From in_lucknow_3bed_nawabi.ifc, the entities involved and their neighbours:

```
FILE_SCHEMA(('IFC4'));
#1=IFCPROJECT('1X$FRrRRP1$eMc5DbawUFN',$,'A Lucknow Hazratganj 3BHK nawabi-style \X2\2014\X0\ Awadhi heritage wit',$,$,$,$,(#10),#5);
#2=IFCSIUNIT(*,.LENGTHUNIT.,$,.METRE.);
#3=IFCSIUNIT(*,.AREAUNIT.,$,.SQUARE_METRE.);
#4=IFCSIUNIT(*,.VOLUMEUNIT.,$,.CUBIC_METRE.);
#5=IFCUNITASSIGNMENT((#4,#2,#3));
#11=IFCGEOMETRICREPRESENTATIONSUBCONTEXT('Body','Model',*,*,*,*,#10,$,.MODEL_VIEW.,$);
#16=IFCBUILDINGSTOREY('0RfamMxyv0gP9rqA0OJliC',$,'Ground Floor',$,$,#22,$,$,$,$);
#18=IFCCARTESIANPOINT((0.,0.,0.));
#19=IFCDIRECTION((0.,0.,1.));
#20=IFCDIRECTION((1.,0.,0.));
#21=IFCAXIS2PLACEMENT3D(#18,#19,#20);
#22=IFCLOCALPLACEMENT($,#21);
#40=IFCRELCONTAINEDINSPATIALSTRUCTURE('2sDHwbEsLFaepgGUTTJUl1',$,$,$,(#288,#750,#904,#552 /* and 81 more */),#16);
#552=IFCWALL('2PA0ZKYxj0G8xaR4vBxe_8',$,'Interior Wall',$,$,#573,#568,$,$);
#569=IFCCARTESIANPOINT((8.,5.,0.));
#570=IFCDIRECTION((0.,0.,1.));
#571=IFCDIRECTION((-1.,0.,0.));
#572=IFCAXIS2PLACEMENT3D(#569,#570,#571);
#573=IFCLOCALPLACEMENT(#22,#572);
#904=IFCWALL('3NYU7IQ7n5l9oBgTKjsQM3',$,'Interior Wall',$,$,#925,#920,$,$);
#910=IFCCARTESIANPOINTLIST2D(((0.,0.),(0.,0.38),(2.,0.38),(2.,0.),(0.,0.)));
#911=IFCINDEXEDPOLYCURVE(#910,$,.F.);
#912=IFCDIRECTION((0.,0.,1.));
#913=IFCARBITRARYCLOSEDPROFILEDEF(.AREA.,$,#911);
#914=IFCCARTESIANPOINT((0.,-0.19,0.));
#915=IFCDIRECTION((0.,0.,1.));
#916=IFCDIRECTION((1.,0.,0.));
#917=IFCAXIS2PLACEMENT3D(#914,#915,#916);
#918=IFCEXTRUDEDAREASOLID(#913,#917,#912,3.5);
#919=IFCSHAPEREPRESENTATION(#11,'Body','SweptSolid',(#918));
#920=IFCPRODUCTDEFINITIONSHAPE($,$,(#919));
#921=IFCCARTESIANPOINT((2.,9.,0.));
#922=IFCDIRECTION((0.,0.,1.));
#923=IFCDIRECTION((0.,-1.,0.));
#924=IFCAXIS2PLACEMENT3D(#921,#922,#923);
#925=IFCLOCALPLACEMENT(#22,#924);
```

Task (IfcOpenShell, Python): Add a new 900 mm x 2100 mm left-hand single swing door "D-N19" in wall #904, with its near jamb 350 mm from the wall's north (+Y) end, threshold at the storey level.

```python
import numpy as np
import ifcopenshell
import ifcopenshell.api.feature
import ifcopenshell.api.geometry
import ifcopenshell.api.root
import ifcopenshell.api.spatial
import ifcopenshell.geom
import ifcopenshell.util.element
import ifcopenshell.util.placement
import ifcopenshell.util.representation
import ifcopenshell.util.shape
import ifcopenshell.util.unit

model = ifcopenshell.open("in_lucknow_3bed_nawabi.ifc")
unit_scale = ifcopenshell.util.unit.calculate_unit_scale(model)
settings = ifcopenshell.geom.settings()


def volume(element):
    """Net volume in cubic metres, openings subtracted."""
    shape = ifcopenshell.geom.create_shape(settings, element)
    return ifcopenshell.util.shape.get_volume(shape.geometry)


wall = model.by_guid("3NYU7IQ7n5l9oBgTKjsQM3")
storey = ifcopenshell.util.element.get_container(wall, ifc_class="IfcBuildingStorey")
context = ifcopenshell.util.representation.get_context(model, "Model", "Body", "MODEL_VIEW")
before = volume(wall)

width, height, from_end, sill = 0.9, 2.1, 0.35, 0.0  # metres

# The wall runs along its own X axis, and the end named is its -X end.
wall_shape = ifcopenshell.geom.create_shape(settings, wall)
x, y, z = ifcopenshell.util.shape.get_vertices(wall_shape.geometry).T
start = x.min() + from_end
face, thickness = float(y.min()), float(y.max() - y.min())
wall_matrix = ifcopenshell.util.placement.get_local_placement(wall.ObjectPlacement)
level = ifcopenshell.util.placement.get_local_placement(storey.ObjectPlacement)[2, 3]


def in_wall(x, y):
    """Placement at x, y metres in the wall's axes, at sill height."""
    matrix = wall_matrix.copy()
    matrix[:, 3] = wall_matrix @ np.array([x / unit_scale, y / unit_scale, 0.0, 1.0])
    matrix[2, 3] = level + sill / unit_scale
    return matrix


# Opening: a box that overshoots both wall faces by 50 mm.
opening = ifcopenshell.api.root.create_entity(model, ifc_class="IfcOpeningElement", predefined_type="OPENING")
box = ifcopenshell.api.geometry.add_wall_representation(
    model, context=context, length=width, height=height, thickness=thickness + 0.1
)
ifcopenshell.api.geometry.assign_representation(model, product=opening, representation=box)
ifcopenshell.api.geometry.edit_object_placement(model, product=opening, matrix=in_wall(start, face - 0.05), is_si=False)
ifcopenshell.api.feature.add_feature(model, feature=opening, element=wall)

door = ifcopenshell.api.root.create_entity(model, ifc_class="IfcDoor", name="D-N19", predefined_type="DOOR")
door.OverallWidth, door.OverallHeight = width / unit_scale, height / unit_scale
door.OperationType = "SINGLE_SWING_LEFT"
body = ifcopenshell.api.geometry.add_door_representation(
    model,
    context=context,
    overall_width=door.OverallWidth,
    overall_height=door.OverallHeight,
    operation_type="SINGLE_SWING_LEFT",
    lining_properties={"LiningDepth": thickness / unit_scale, "ThresholdDepth": thickness / unit_scale},
)
ifcopenshell.api.geometry.assign_representation(model, product=door, representation=body)
ifcopenshell.api.spatial.assign_container(model, products=[door], relating_structure=storey)
ifcopenshell.api.feature.add_filling(model, opening=opening, element=door)

# The lining spans the wall, so the door starts at the wall face.
ifcopenshell.api.geometry.edit_object_placement(model, product=door, matrix=in_wall(start, face), is_si=False)

after = volume(wall)

print(f"wall volume {before:.3f} -> {after:.3f} m3")

model.write("in_lucknow_3bed_nawabi_rev.ifc")
```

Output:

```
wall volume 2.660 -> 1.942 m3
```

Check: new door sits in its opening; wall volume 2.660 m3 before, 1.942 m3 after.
